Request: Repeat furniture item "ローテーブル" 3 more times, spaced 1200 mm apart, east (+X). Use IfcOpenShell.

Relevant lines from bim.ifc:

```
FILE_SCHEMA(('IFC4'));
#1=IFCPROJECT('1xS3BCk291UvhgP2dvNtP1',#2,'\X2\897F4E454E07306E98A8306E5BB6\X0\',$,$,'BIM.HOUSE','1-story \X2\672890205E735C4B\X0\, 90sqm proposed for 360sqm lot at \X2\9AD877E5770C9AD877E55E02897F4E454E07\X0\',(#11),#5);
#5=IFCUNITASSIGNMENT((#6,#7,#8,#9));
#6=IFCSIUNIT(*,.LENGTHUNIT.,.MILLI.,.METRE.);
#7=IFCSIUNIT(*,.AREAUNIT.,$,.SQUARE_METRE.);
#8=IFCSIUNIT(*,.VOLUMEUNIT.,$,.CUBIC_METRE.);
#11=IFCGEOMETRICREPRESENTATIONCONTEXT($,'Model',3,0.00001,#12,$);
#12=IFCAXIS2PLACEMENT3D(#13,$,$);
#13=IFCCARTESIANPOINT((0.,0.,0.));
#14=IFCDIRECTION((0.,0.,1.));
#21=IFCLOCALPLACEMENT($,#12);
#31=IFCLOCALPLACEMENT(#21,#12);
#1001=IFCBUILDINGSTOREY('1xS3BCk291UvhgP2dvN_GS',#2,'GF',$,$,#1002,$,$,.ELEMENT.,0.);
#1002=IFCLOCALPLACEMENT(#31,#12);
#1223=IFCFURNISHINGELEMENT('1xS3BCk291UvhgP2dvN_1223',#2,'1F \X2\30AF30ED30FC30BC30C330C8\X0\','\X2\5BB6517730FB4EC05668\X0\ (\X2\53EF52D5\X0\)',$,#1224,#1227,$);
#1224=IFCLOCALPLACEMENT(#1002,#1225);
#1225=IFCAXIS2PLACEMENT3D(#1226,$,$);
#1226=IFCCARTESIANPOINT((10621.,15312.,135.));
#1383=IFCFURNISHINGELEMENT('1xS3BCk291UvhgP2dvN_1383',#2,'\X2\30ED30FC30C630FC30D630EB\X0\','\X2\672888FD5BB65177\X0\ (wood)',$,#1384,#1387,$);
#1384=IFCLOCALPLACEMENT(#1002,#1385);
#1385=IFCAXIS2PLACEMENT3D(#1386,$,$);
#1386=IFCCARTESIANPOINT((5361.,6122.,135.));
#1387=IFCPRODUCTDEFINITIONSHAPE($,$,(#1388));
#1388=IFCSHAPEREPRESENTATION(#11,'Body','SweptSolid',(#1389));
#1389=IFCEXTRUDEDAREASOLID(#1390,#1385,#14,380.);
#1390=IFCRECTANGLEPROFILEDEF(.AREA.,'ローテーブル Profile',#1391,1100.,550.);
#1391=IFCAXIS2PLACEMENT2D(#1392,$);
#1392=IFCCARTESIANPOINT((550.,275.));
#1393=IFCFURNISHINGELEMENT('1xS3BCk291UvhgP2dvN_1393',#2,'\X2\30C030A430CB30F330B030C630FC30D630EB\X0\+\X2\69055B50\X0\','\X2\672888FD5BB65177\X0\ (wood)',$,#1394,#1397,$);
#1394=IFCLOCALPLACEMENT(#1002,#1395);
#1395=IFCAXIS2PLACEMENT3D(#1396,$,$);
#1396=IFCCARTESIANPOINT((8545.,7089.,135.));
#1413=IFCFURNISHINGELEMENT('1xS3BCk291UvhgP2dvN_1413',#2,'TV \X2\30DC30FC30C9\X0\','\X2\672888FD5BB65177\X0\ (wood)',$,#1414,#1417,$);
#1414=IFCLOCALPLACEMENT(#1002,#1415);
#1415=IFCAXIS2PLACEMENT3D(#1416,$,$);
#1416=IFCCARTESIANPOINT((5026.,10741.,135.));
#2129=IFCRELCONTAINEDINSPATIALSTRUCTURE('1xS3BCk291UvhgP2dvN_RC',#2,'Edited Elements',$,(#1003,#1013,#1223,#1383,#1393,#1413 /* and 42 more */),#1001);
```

```python
import numpy as np
import ifcopenshell
import ifcopenshell.api.geometry
import ifcopenshell.api.root
import ifcopenshell.util.element
import ifcopenshell.util.placement

model = ifcopenshell.open("bim.ifc")


def reuse_history(source, copy):
    """copy_class also copies each property set's owner history, people and application; keep the originals."""
    for rel in copy.IsDefinedBy:
        if rel.is_a("IfcRelDefinesByProperties") and (history := rel.RelatingPropertyDefinition.OwnerHistory):
            rel.RelatingPropertyDefinition.OwnerHistory = source.OwnerHistory
            ifcopenshell.util.element.remove_deep2(model, history)


source = model.by_id(1383)
base = ifcopenshell.util.placement.get_local_placement(source.ObjectPlacement)
step = np.array([1.0, 0.0, 0.0]) * 1200.0

for i in range(1, 4):
    copy = ifcopenshell.api.root.copy_class(model, product=source)
    copy.Representation = ifcopenshell.util.element.copy_deep(
        model, source.Representation, exclude=["IfcGeometricRepresentationContext", "IfcRepresentationMap"]
    )
    reuse_history(source, copy)
    matrix = base.copy()
    matrix[:3, 3] += i * step
    print("added at", matrix[:3, 3].round(3) + 0.0)
    ifcopenshell.api.geometry.edit_object_placement(model, product=copy, matrix=matrix, is_si=False)

model.write("bim_v2.ifc")
```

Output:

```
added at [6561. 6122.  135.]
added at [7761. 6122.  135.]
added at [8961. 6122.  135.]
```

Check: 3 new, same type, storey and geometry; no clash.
